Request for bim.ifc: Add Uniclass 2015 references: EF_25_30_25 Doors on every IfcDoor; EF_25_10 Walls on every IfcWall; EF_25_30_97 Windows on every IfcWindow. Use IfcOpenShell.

First a look at what the model holds.

```python
import ifcopenshell

model = ifcopenshell.open("bim.ifc")
print(model.schema)
print("classifications:", [c.Name for c in model.by_type("IfcClassification")])
for ifc_class in ("IfcDoor", "IfcRoof", "IfcStair", "IfcWall", "IfcWindow"):
    print(ifc_class, len(model.by_type(ifc_class)))
```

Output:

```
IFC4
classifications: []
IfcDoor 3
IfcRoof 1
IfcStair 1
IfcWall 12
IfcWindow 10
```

```python
import ifcopenshell
import ifcopenshell.api.classification

model = ifcopenshell.open("bim.ifc")

system = ifcopenshell.api.classification.add_classification(model, classification="Uniclass 2015")

codes = {
    "IfcDoor": ("EF_25_30_25", "Doors"),
    "IfcWall": ("EF_25_10", "Walls"),
    "IfcWindow": ("EF_25_30_97", "Windows"),
}
for ifc_class, (code, name) in codes.items():
    products = model.by_type(ifc_class)
    ifcopenshell.api.classification.add_reference(
        model, products=products, classification=system, identification=code, name=name
    )
    print(code, len(products))

model.write("bim_v2.ifc")
```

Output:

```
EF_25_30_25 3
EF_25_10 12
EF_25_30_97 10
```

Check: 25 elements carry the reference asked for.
